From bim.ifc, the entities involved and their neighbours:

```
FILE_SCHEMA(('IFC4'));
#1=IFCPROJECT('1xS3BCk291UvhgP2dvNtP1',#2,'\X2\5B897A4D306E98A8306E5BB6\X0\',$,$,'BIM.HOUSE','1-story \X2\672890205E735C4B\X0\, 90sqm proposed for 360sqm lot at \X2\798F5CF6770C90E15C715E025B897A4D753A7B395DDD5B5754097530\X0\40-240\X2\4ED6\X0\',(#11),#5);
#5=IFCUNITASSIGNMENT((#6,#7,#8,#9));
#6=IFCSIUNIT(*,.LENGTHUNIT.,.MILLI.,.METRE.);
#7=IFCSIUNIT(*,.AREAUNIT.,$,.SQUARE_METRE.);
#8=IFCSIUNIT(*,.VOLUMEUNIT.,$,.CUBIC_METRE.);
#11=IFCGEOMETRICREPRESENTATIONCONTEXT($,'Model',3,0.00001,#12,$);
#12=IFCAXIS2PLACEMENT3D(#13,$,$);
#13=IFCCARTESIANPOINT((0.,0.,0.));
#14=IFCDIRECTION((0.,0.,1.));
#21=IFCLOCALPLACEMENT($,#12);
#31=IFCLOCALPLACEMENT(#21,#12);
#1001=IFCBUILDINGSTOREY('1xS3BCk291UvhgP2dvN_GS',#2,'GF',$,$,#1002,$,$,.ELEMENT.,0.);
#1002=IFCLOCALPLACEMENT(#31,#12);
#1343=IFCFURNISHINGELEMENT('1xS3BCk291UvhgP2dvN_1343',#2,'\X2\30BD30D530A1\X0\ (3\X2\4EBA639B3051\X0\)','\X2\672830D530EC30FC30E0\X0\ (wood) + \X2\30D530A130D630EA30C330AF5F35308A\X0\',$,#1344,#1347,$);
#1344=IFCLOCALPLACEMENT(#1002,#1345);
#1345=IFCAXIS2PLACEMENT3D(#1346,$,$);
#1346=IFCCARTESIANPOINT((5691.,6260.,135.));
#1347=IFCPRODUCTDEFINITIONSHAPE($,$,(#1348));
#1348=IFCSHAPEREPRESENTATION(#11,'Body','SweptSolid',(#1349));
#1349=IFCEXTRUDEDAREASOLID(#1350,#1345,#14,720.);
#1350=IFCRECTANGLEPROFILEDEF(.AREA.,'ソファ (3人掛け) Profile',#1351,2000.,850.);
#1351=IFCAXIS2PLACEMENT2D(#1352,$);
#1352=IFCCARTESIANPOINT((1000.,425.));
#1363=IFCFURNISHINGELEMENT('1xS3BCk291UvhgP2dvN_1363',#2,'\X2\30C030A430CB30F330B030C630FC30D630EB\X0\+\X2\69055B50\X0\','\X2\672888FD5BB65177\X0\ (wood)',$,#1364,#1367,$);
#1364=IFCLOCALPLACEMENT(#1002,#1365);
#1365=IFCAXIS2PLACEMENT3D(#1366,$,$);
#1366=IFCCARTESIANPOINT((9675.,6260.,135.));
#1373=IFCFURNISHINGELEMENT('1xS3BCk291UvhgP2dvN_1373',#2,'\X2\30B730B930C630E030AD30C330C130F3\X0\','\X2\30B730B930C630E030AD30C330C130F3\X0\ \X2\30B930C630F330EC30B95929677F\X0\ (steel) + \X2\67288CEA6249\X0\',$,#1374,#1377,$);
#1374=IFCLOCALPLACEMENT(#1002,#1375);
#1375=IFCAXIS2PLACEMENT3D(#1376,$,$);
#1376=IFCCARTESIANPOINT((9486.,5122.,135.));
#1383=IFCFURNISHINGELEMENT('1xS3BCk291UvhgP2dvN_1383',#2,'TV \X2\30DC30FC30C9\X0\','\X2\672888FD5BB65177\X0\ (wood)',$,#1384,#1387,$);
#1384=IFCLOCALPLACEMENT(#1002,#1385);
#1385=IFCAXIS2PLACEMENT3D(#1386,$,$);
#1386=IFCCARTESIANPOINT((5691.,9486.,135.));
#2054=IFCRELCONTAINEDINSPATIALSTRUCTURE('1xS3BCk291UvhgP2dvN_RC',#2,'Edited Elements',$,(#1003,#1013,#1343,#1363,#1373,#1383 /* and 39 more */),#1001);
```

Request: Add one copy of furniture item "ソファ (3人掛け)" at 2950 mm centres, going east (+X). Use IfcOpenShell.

```python
import numpy as np
import ifcopenshell
import ifcopenshell.api.geometry
import ifcopenshell.api.root
import ifcopenshell.util.element
import ifcopenshell.util.placement
import ifcopenshell.util.unit

model = ifcopenshell.open("bim.ifc")
unit_scale = ifcopenshell.util.unit.calculate_unit_scale(model)


def reuse_history(source, copy):
    """copy_class also copies each property set's owner history, people and application; keep the originals."""
    for rel in copy.IsDefinedBy:
        if rel.is_a("IfcRelDefinesByProperties") and (history := rel.RelatingPropertyDefinition.OwnerHistory):
            rel.RelatingPropertyDefinition.OwnerHistory = source.OwnerHistory
            ifcopenshell.util.element.remove_deep2(model, history)


source = model.by_guid("1xS3BCk291UvhgP2dvN_1343")
base = ifcopenshell.util.placement.get_local_placement(source.ObjectPlacement)
step = np.array([1.0, 0.0, 0.0]) * 2.95 / unit_scale

for i in range(1, 2):
    copy = ifcopenshell.api.root.copy_class(model, product=source)
    copy.Representation = ifcopenshell.util.element.copy_deep(
        model, source.Representation, exclude=["IfcGeometricRepresentationContext", "IfcRepresentationMap"]
    )
    reuse_history(source, copy)
    matrix = base.copy()
    matrix[:3, 3] += i * step
    print("added at", matrix[:3, 3].round(3) + 0.0)
    ifcopenshell.api.geometry.edit_object_placement(model, product=copy, matrix=matrix, is_si=False)

model.write("bim-out.ifc")
```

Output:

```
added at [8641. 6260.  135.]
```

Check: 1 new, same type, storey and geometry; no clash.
